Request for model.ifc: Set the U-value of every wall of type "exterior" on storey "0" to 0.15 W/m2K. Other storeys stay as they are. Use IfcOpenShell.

First a look at what the model holds.

```python
import ifcopenshell
import ifcopenshell.util.element

model = ifcopenshell.open("model.ifc")
print(model.schema)
storey = next(s for s in model.by_type("IfcBuildingStorey") if s.Name == "0")
walls = [e for e in ifcopenshell.util.element.get_decomposition(storey) if e.is_a("IfcWall")]
seen = {}
for e in walls:
    element_type = ifcopenshell.util.element.get_type(e)
    key = (element_type.Name if element_type != e and element_type else None, ifcopenshell.util.element.get_pset(e, "Pset_WallCommon", "ThermalTransmittance"))
    seen[key] = seen.get(key, 0) + 1
for (name, value), count in sorted(seen.items(), key=str):
    print(count, "x", name, "|", value)
```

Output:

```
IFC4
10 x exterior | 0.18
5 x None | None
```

```python
import ifcopenshell
import ifcopenshell.api.pset
import ifcopenshell.util.element

model = ifcopenshell.open("model.ifc")

storey = next(s for s in model.by_type("IfcBuildingStorey") if s.Name == "0")
walls = [e for e in ifcopenshell.util.element.get_decomposition(storey) if e.is_a("IfcWall")]

count = 0
for e in walls:
    element_type = ifcopenshell.util.element.get_type(e)
    if element_type in (None, e) or element_type.Name != "exterior":
        continue
    # add_pset returns the element's existing set when there is one.
    pset = ifcopenshell.api.pset.add_pset(model, product=e, name="Pset_WallCommon")
    ifcopenshell.api.pset.edit_pset(model, pset=pset, properties={"ThermalTransmittance": 0.15})
    count += 1

print(count, "walls updated")

model.write("model_edited.ifc")
```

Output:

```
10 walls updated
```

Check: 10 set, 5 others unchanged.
